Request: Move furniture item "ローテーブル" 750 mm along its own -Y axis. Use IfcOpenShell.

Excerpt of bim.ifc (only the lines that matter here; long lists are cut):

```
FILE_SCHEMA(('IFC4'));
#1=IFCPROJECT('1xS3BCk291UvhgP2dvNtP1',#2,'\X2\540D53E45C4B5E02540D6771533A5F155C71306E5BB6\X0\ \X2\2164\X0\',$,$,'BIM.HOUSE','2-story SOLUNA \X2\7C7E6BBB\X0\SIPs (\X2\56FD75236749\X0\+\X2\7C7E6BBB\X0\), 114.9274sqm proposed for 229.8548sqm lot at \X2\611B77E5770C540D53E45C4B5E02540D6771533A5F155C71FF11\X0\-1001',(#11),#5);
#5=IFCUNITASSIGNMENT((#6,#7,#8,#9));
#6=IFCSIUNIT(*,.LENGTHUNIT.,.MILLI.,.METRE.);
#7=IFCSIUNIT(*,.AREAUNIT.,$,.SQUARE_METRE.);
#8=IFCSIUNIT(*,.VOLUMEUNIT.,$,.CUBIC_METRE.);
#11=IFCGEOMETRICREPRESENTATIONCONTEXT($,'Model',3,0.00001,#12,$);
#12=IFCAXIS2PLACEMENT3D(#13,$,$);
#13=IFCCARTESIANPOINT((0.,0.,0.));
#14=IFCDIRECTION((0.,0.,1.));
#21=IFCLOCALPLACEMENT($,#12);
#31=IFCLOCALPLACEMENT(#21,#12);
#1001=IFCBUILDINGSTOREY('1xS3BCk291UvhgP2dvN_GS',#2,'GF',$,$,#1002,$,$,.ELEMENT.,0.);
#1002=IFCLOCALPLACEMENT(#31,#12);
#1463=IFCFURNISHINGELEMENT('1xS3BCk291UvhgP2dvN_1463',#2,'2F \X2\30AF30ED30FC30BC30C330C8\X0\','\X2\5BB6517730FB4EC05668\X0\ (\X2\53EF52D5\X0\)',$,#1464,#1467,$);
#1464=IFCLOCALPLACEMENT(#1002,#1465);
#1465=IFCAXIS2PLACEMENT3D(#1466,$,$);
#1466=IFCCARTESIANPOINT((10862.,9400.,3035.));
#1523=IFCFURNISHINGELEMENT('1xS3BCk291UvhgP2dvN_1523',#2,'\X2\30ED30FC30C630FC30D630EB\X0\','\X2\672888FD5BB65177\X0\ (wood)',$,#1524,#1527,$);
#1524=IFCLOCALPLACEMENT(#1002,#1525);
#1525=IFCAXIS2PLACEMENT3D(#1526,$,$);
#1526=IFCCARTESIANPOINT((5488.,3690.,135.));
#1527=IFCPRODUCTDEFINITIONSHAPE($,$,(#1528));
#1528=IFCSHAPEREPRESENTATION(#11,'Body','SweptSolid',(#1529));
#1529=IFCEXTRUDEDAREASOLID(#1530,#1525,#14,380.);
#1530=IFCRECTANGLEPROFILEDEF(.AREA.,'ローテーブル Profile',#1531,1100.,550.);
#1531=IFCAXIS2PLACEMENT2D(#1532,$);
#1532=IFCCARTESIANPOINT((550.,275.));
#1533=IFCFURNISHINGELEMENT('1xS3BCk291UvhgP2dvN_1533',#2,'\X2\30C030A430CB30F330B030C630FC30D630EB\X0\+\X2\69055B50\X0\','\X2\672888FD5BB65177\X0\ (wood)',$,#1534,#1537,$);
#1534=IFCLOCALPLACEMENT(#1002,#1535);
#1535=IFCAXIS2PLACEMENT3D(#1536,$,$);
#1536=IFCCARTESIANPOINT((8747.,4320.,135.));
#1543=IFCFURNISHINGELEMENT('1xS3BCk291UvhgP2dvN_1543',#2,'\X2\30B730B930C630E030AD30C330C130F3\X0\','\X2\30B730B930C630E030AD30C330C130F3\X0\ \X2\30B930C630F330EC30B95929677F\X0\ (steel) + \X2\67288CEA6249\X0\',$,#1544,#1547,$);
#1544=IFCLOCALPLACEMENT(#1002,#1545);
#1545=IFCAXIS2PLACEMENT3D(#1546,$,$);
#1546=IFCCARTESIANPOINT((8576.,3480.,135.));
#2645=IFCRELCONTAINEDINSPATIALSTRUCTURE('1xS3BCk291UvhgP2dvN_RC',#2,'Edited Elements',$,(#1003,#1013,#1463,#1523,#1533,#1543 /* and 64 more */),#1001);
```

```python
import ifcopenshell
import ifcopenshell.api.geometry
import ifcopenshell.util.placement
import ifcopenshell.util.unit

model = ifcopenshell.open("bim.ifc")
unit_scale = ifcopenshell.util.unit.calculate_unit_scale(model)

item = model.by_guid("1xS3BCk291UvhgP2dvN_1523")
matrix = ifcopenshell.util.placement.get_local_placement(item.ObjectPlacement)
matrix[:3, 3] -= matrix[:3, 1] * 0.75 / unit_scale
ifcopenshell.api.geometry.edit_object_placement(model, product=item, matrix=matrix, is_si=False)

print(ifcopenshell.util.placement.get_local_placement(item.ObjectPlacement).round(3) + 0.0)

model.write("bim_updated.ifc")
```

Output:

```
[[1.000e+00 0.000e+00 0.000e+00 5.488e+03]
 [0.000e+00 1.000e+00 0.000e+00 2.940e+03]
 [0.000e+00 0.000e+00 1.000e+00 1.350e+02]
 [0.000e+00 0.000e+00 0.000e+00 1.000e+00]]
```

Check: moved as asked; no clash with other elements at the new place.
